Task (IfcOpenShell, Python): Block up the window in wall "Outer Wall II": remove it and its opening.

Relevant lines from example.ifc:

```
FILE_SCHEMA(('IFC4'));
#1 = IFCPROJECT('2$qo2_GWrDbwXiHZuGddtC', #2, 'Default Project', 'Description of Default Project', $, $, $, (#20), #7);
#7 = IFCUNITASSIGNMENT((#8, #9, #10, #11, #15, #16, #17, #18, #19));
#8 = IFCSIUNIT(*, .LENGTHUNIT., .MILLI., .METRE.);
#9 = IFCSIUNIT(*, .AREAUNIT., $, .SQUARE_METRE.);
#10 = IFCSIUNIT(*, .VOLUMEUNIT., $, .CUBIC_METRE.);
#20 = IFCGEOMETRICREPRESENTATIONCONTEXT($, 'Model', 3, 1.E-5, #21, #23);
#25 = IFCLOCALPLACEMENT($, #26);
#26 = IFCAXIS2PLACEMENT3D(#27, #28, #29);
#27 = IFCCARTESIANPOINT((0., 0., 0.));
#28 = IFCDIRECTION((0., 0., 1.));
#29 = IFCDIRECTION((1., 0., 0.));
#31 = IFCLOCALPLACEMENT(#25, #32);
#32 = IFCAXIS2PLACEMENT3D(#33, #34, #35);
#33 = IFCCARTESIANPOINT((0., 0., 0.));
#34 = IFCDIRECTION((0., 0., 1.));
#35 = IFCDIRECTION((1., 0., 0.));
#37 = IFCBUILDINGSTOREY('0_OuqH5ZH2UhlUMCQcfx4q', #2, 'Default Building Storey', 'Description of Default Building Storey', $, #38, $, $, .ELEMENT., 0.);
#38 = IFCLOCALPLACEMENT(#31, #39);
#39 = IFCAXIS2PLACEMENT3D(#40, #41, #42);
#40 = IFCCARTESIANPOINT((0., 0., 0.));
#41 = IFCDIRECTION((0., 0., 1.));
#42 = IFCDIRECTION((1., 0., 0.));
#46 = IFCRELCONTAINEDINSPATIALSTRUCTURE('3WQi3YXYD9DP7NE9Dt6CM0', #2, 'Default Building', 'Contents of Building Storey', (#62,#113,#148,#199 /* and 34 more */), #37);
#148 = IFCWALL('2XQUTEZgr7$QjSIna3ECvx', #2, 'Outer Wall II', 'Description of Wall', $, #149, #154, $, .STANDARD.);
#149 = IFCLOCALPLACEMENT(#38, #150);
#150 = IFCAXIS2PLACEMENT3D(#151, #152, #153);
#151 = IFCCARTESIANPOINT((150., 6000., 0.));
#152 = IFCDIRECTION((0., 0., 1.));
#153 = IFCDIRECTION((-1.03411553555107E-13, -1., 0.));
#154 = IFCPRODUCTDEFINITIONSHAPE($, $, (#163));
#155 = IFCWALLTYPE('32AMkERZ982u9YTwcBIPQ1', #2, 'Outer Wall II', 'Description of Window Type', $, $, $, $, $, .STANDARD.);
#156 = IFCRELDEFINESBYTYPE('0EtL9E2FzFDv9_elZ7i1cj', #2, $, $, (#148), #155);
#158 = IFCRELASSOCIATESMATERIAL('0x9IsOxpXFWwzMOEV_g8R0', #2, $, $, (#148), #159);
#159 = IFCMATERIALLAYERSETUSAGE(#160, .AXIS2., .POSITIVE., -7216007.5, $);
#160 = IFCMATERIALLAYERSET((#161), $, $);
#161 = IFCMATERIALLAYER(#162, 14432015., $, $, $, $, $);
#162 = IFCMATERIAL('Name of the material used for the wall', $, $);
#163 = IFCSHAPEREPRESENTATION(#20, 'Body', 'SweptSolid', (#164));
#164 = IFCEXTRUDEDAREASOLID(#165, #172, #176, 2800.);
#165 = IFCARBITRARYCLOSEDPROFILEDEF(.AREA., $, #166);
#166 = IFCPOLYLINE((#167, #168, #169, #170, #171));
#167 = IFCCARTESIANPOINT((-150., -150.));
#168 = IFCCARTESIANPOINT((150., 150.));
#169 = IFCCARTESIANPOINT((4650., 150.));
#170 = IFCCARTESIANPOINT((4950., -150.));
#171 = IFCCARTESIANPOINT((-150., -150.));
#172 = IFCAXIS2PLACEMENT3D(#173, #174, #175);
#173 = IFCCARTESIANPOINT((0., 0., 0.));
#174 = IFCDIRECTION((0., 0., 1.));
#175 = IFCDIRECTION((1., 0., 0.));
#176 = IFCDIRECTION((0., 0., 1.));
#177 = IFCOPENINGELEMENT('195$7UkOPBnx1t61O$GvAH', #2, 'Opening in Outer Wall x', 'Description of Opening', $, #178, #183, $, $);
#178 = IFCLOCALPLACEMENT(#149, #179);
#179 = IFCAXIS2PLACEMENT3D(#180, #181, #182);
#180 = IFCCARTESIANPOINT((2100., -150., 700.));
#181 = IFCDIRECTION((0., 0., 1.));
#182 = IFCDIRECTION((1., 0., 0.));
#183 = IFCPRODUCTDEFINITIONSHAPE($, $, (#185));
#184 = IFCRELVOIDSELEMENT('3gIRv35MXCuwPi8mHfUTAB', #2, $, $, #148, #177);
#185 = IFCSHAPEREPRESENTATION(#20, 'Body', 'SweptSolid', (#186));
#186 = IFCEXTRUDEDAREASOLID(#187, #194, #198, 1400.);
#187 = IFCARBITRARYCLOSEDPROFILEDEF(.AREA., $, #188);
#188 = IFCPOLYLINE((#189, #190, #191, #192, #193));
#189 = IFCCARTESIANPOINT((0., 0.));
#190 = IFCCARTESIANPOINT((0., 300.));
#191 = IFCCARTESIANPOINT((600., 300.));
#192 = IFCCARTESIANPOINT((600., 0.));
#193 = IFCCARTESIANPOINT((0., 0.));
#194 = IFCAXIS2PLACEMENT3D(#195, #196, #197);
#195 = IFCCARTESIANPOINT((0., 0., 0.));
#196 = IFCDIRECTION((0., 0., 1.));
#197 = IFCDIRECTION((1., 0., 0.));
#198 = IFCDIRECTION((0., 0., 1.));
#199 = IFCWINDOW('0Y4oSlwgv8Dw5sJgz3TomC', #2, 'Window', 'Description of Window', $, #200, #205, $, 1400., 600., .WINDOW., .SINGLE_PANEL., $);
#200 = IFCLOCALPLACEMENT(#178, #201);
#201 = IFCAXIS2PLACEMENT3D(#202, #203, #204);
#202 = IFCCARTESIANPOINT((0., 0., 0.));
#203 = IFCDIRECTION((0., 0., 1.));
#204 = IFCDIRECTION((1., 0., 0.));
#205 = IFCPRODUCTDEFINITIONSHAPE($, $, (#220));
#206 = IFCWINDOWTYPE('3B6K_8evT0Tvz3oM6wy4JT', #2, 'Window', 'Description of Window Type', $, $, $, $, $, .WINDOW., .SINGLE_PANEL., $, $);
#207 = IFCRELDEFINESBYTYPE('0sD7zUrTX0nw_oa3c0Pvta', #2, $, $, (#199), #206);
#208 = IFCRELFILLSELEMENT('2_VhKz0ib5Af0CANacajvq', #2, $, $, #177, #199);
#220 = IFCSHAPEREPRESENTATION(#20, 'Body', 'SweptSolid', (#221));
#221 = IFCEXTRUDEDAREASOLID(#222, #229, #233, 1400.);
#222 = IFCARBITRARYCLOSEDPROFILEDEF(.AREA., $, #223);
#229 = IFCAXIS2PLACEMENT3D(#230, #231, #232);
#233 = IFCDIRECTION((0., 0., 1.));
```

```python
import ifcopenshell
import ifcopenshell.api.feature
import ifcopenshell.api.root
import ifcopenshell.geom
import ifcopenshell.util.shape

model = ifcopenshell.open("example.ifc")
settings = ifcopenshell.geom.settings()


def volume(element):
    """Net volume in cubic metres, openings subtracted."""
    shape = ifcopenshell.geom.create_shape(settings, element)
    return ifcopenshell.util.shape.get_volume(shape.geometry)


window = model.by_guid("0Y4oSlwgv8Dw5sJgz3TomC")
opening = window.FillsVoids[0].RelatingOpeningElement
wall = opening.VoidsElements[0].RelatingBuildingElement
before = volume(wall)

ifcopenshell.api.root.remove_product(model, product=window)
ifcopenshell.api.feature.remove_feature(model, feature=opening)

after = volume(wall)

print(f"wall volume {before:.3f} -> {after:.3f} m3")

model.write("example_v2.ifc")
```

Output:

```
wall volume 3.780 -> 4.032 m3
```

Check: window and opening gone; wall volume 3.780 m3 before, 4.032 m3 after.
